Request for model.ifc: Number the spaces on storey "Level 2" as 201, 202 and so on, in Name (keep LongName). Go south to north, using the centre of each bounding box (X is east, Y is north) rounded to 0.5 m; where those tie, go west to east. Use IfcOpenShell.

First a look at what the model holds.

```python
import ifcopenshell
import ifcopenshell.util.element
import ifcopenshell.util.placement

model = ifcopenshell.open("model.ifc")
print(model.schema)
storey = next(s for s in model.by_type("IfcBuildingStorey") if s.Name == "Level 2")
spaces = [e for e in ifcopenshell.util.element.get_decomposition(storey) if e.is_a("IfcSpace")]
for e in sorted(spaces, key=lambda e: e.id()):
    origin = ifcopenshell.util.placement.get_local_placement(e.ObjectPlacement)[:3, 3]
    print(e.id(), e.Name, e.LongName, origin.round(2) + 0.0, sep=" | ")
```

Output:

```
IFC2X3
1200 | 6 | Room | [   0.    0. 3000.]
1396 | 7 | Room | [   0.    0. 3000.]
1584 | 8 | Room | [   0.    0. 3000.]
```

```python
import ifcopenshell
import ifcopenshell.geom
import ifcopenshell.util.element
import ifcopenshell.util.shape

model = ifcopenshell.open("model.ifc")
settings = ifcopenshell.geom.settings()
settings.set("use-world-coords", True)


def centre(element):
    shape = ifcopenshell.geom.create_shape(settings, element)
    return ifcopenshell.util.shape.get_bbox_centroid(shape.geometry)


storey = next(s for s in model.by_type("IfcBuildingStorey") if s.Name == "Level 2")
spaces = [e for e in ifcopenshell.util.element.get_decomposition(storey) if e.is_a("IfcSpace")]

# Insertion points can sit at a corner or the storey origin, so sort by the geometry (in metres).
centres = {e: centre(e) for e in spaces}
spaces.sort(key=lambda e: (round(centres[e][1] / 0.5), centres[e][0]))

for i, e in enumerate(spaces, start=1):
    number = f"2{i:02d}"
    e.Name = number
    print(e.id(), number)

model.write("model_v2.ifc")
```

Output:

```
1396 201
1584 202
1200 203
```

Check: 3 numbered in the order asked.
